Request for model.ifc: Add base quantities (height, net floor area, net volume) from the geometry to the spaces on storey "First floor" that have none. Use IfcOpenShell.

First a look at what the model holds.

```python
import ifcopenshell
import ifcopenshell.util.element
import ifcopenshell.util.unit

model = ifcopenshell.open("model.ifc")
print(model.schema)
for unit_type in ("LENGTHUNIT", "AREAUNIT", "VOLUMEUNIT"):
    print(unit_type, ifcopenshell.util.unit.calculate_unit_scale(model, unit_type))
storey = next(s for s in model.by_type("IfcBuildingStorey") if s.Name == "First floor")
spaces = [e for e in ifcopenshell.util.element.get_decomposition(storey) if e.is_a("IfcSpace")]
for e in sorted(spaces, key=lambda e: e.id()):
    print(e.id(), e.is_a(), e.Name, list(ifcopenshell.util.element.get_psets(e, qtos_only=True)), sep=" | ")
```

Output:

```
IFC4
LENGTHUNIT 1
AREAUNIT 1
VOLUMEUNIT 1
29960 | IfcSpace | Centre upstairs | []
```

```python
import ifcopenshell
import ifcopenshell.api.pset
import ifcopenshell.geom
import ifcopenshell.util.element
import ifcopenshell.util.shape
import ifcopenshell.util.unit

model = ifcopenshell.open("model.ifc")
unit_scale = ifcopenshell.util.unit.calculate_unit_scale(model)
area_scale = ifcopenshell.util.unit.calculate_unit_scale(model, "AREAUNIT")
volume_scale = ifcopenshell.util.unit.calculate_unit_scale(model, "VOLUMEUNIT")
settings = ifcopenshell.geom.settings()

storey = next(s for s in model.by_type("IfcBuildingStorey") if s.Name == "First floor")
spaces = [e for e in ifcopenshell.util.element.get_decomposition(storey) if e.is_a("IfcSpace")]

for e in sorted(spaces, key=lambda e: e.id()):
    if ifcopenshell.util.element.get_psets(e, qtos_only=True, should_inherit=False):
        continue
    # Geometry comes back in metres, in the element's own axes.
    shape = ifcopenshell.geom.create_shape(settings, e)
    values = {
        "Height": ifcopenshell.util.shape.get_z(shape.geometry) / unit_scale,
        "NetFloorArea": ifcopenshell.util.shape.get_footprint_area(shape.geometry) / area_scale,
        "NetVolume": ifcopenshell.util.shape.get_volume(shape.geometry) / volume_scale,
    }
    qto = ifcopenshell.api.pset.add_qto(model, product=e, name="Qto_SpaceBaseQuantities")
    ifcopenshell.api.pset.edit_qto(model, qto=qto, properties=values)
    print(e.id(), {k: round(v, 3) for k, v in values.items()})

model.write("model_rev.ifc")
```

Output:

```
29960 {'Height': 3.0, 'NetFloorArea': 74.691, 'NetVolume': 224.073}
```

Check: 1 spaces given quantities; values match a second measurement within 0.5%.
